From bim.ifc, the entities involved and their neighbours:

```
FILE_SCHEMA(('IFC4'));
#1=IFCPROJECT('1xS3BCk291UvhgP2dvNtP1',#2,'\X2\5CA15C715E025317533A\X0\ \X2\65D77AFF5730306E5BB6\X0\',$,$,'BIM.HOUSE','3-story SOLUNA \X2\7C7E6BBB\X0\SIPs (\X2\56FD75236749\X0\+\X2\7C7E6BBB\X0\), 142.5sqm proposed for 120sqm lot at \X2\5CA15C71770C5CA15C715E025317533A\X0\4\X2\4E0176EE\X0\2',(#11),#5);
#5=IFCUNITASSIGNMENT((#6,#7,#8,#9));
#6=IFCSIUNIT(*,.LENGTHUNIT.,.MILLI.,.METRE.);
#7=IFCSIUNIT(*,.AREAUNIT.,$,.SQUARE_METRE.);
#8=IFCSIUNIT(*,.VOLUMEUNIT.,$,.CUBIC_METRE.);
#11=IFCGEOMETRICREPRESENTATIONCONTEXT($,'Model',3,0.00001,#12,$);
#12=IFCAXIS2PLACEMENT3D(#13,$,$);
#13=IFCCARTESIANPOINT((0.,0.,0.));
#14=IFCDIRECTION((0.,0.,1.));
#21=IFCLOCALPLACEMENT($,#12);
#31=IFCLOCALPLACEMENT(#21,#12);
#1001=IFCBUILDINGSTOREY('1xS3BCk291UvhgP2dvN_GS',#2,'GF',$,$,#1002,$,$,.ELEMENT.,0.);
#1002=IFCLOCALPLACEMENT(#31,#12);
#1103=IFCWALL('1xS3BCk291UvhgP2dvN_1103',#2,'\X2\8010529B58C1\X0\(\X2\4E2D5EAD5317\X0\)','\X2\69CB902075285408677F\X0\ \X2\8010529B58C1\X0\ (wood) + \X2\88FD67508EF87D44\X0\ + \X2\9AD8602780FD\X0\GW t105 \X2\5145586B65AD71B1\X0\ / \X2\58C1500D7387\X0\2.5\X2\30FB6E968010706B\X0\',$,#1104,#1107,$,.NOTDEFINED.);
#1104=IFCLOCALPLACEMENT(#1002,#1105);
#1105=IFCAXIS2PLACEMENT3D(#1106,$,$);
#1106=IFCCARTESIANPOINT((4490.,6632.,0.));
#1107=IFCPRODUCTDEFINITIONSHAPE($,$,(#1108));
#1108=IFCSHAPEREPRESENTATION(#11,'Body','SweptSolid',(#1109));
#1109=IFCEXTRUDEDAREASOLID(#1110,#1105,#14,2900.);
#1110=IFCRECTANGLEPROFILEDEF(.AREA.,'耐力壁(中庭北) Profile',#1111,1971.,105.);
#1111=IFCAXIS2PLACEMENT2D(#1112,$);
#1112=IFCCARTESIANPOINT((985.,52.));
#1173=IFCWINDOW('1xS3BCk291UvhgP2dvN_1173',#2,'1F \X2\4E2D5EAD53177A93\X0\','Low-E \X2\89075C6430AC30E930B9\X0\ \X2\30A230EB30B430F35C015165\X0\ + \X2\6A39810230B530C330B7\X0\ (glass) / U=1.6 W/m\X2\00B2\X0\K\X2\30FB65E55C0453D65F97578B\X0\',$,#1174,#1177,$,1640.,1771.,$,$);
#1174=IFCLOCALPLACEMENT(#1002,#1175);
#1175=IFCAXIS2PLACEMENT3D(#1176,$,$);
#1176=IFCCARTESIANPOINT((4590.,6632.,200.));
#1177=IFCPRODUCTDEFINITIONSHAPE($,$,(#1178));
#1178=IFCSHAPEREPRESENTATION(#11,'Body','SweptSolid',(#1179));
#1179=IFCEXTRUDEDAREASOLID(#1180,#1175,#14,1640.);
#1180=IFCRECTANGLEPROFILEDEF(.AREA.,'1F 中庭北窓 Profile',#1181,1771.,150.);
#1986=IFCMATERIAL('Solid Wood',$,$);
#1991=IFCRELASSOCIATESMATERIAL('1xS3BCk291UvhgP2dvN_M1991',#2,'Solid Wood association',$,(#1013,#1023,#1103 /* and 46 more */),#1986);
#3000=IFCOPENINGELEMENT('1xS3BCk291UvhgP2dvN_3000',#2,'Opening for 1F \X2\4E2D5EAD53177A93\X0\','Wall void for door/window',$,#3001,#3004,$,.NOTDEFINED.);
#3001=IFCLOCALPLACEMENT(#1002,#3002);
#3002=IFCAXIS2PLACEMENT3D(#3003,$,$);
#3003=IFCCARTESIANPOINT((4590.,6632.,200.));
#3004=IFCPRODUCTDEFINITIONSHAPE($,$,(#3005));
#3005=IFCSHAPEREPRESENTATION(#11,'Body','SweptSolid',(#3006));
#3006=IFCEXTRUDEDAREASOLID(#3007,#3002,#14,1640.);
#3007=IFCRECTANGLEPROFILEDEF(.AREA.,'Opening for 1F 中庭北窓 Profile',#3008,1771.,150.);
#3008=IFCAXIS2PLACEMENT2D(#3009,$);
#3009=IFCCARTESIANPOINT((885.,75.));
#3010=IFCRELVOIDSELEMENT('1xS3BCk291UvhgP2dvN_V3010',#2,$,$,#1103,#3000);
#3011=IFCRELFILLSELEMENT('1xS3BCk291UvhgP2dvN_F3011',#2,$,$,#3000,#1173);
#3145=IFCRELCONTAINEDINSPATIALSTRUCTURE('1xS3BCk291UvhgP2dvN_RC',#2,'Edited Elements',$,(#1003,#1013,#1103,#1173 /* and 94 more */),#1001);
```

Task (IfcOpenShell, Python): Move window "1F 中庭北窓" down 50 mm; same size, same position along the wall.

```python
import numpy as np
import ifcopenshell
import ifcopenshell.api.geometry
import ifcopenshell.util.placement
import ifcopenshell.util.unit

model = ifcopenshell.open("bim.ifc")
unit_scale = ifcopenshell.util.unit.calculate_unit_scale(model)

window = model.by_guid("1xS3BCk291UvhgP2dvN_1173")
opening = window.FillsVoids[0].RelatingOpeningElement
dz = -0.05 / unit_scale

shift = np.array([0.0, 0.0, dz])
# The window is not placed relative to its opening, so move both.
for product in (opening, window):
    matrix = ifcopenshell.util.placement.get_local_placement(product.ObjectPlacement)
    matrix[:3, 3] += shift
    ifcopenshell.api.geometry.edit_object_placement(model, product=product, matrix=matrix, is_si=False)

print(f"moved by {dz * unit_scale:+.3f} m")

model.write("bim_updated.ifc")
```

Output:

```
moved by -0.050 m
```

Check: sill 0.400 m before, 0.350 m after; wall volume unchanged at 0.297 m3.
